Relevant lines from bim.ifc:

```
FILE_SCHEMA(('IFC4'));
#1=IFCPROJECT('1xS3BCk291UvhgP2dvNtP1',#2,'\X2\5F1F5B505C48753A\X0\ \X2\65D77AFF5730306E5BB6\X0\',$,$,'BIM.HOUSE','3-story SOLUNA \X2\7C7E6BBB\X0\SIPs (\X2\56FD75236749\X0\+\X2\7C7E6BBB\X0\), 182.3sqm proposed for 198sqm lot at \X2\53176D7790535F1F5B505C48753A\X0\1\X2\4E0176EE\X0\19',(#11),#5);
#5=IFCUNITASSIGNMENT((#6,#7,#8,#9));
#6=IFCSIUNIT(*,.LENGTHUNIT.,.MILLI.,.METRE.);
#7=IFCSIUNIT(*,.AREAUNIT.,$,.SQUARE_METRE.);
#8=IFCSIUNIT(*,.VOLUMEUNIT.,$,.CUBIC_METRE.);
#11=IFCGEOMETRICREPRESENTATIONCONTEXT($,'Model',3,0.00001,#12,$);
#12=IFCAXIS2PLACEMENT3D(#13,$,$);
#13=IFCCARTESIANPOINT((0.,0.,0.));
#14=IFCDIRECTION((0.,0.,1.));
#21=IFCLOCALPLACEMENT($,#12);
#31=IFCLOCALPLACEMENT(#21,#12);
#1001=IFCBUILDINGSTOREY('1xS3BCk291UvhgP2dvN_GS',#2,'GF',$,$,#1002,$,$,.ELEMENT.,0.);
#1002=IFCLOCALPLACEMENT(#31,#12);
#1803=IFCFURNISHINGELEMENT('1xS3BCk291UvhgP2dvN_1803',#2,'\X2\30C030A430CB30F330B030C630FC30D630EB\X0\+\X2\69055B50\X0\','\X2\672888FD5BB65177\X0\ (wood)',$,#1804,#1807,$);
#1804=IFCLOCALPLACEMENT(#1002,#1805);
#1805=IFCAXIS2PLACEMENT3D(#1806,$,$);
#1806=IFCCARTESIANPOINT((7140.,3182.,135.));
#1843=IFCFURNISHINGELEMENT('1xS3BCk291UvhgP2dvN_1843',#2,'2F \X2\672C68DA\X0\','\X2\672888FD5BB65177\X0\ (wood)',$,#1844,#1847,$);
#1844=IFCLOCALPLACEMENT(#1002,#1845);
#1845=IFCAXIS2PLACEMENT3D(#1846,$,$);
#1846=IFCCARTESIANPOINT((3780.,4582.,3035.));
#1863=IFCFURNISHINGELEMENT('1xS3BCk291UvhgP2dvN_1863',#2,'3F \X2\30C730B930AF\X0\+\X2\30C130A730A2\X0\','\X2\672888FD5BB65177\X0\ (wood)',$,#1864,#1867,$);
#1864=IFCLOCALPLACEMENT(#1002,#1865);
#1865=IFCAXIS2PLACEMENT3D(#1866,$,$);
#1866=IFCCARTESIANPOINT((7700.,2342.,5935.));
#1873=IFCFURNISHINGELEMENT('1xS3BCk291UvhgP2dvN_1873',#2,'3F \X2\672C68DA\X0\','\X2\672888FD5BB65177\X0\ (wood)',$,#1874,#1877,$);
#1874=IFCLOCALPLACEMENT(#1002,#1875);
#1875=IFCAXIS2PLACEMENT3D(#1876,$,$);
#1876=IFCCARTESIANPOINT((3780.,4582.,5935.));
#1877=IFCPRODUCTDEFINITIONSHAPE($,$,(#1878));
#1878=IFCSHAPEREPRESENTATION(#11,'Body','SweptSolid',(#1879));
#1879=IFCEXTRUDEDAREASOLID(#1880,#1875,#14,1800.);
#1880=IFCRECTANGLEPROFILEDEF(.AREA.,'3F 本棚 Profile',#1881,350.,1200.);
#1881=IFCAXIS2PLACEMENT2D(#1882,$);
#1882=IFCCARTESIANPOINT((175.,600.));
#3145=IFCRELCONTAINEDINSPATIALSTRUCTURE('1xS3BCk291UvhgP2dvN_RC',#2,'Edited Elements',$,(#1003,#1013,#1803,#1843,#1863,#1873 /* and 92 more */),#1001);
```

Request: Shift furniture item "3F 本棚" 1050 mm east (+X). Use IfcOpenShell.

```python
import ifcopenshell
import ifcopenshell.api.geometry
import ifcopenshell.util.placement
import ifcopenshell.util.unit

model = ifcopenshell.open("bim.ifc")
unit_scale = ifcopenshell.util.unit.calculate_unit_scale(model)

item = model.by_guid("1xS3BCk291UvhgP2dvN_1873")
matrix = ifcopenshell.util.placement.get_local_placement(item.ObjectPlacement)
matrix[0, 3] += 1.05 / unit_scale
ifcopenshell.api.geometry.edit_object_placement(model, product=item, matrix=matrix, is_si=False)

print(ifcopenshell.util.placement.get_local_placement(item.ObjectPlacement).round(3) + 0.0)

model.write("bim_v2.ifc")
```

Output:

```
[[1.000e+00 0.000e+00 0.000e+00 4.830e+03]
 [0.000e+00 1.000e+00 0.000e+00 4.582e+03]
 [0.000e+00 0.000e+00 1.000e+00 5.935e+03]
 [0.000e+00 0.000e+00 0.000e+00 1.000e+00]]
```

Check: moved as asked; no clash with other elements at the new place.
